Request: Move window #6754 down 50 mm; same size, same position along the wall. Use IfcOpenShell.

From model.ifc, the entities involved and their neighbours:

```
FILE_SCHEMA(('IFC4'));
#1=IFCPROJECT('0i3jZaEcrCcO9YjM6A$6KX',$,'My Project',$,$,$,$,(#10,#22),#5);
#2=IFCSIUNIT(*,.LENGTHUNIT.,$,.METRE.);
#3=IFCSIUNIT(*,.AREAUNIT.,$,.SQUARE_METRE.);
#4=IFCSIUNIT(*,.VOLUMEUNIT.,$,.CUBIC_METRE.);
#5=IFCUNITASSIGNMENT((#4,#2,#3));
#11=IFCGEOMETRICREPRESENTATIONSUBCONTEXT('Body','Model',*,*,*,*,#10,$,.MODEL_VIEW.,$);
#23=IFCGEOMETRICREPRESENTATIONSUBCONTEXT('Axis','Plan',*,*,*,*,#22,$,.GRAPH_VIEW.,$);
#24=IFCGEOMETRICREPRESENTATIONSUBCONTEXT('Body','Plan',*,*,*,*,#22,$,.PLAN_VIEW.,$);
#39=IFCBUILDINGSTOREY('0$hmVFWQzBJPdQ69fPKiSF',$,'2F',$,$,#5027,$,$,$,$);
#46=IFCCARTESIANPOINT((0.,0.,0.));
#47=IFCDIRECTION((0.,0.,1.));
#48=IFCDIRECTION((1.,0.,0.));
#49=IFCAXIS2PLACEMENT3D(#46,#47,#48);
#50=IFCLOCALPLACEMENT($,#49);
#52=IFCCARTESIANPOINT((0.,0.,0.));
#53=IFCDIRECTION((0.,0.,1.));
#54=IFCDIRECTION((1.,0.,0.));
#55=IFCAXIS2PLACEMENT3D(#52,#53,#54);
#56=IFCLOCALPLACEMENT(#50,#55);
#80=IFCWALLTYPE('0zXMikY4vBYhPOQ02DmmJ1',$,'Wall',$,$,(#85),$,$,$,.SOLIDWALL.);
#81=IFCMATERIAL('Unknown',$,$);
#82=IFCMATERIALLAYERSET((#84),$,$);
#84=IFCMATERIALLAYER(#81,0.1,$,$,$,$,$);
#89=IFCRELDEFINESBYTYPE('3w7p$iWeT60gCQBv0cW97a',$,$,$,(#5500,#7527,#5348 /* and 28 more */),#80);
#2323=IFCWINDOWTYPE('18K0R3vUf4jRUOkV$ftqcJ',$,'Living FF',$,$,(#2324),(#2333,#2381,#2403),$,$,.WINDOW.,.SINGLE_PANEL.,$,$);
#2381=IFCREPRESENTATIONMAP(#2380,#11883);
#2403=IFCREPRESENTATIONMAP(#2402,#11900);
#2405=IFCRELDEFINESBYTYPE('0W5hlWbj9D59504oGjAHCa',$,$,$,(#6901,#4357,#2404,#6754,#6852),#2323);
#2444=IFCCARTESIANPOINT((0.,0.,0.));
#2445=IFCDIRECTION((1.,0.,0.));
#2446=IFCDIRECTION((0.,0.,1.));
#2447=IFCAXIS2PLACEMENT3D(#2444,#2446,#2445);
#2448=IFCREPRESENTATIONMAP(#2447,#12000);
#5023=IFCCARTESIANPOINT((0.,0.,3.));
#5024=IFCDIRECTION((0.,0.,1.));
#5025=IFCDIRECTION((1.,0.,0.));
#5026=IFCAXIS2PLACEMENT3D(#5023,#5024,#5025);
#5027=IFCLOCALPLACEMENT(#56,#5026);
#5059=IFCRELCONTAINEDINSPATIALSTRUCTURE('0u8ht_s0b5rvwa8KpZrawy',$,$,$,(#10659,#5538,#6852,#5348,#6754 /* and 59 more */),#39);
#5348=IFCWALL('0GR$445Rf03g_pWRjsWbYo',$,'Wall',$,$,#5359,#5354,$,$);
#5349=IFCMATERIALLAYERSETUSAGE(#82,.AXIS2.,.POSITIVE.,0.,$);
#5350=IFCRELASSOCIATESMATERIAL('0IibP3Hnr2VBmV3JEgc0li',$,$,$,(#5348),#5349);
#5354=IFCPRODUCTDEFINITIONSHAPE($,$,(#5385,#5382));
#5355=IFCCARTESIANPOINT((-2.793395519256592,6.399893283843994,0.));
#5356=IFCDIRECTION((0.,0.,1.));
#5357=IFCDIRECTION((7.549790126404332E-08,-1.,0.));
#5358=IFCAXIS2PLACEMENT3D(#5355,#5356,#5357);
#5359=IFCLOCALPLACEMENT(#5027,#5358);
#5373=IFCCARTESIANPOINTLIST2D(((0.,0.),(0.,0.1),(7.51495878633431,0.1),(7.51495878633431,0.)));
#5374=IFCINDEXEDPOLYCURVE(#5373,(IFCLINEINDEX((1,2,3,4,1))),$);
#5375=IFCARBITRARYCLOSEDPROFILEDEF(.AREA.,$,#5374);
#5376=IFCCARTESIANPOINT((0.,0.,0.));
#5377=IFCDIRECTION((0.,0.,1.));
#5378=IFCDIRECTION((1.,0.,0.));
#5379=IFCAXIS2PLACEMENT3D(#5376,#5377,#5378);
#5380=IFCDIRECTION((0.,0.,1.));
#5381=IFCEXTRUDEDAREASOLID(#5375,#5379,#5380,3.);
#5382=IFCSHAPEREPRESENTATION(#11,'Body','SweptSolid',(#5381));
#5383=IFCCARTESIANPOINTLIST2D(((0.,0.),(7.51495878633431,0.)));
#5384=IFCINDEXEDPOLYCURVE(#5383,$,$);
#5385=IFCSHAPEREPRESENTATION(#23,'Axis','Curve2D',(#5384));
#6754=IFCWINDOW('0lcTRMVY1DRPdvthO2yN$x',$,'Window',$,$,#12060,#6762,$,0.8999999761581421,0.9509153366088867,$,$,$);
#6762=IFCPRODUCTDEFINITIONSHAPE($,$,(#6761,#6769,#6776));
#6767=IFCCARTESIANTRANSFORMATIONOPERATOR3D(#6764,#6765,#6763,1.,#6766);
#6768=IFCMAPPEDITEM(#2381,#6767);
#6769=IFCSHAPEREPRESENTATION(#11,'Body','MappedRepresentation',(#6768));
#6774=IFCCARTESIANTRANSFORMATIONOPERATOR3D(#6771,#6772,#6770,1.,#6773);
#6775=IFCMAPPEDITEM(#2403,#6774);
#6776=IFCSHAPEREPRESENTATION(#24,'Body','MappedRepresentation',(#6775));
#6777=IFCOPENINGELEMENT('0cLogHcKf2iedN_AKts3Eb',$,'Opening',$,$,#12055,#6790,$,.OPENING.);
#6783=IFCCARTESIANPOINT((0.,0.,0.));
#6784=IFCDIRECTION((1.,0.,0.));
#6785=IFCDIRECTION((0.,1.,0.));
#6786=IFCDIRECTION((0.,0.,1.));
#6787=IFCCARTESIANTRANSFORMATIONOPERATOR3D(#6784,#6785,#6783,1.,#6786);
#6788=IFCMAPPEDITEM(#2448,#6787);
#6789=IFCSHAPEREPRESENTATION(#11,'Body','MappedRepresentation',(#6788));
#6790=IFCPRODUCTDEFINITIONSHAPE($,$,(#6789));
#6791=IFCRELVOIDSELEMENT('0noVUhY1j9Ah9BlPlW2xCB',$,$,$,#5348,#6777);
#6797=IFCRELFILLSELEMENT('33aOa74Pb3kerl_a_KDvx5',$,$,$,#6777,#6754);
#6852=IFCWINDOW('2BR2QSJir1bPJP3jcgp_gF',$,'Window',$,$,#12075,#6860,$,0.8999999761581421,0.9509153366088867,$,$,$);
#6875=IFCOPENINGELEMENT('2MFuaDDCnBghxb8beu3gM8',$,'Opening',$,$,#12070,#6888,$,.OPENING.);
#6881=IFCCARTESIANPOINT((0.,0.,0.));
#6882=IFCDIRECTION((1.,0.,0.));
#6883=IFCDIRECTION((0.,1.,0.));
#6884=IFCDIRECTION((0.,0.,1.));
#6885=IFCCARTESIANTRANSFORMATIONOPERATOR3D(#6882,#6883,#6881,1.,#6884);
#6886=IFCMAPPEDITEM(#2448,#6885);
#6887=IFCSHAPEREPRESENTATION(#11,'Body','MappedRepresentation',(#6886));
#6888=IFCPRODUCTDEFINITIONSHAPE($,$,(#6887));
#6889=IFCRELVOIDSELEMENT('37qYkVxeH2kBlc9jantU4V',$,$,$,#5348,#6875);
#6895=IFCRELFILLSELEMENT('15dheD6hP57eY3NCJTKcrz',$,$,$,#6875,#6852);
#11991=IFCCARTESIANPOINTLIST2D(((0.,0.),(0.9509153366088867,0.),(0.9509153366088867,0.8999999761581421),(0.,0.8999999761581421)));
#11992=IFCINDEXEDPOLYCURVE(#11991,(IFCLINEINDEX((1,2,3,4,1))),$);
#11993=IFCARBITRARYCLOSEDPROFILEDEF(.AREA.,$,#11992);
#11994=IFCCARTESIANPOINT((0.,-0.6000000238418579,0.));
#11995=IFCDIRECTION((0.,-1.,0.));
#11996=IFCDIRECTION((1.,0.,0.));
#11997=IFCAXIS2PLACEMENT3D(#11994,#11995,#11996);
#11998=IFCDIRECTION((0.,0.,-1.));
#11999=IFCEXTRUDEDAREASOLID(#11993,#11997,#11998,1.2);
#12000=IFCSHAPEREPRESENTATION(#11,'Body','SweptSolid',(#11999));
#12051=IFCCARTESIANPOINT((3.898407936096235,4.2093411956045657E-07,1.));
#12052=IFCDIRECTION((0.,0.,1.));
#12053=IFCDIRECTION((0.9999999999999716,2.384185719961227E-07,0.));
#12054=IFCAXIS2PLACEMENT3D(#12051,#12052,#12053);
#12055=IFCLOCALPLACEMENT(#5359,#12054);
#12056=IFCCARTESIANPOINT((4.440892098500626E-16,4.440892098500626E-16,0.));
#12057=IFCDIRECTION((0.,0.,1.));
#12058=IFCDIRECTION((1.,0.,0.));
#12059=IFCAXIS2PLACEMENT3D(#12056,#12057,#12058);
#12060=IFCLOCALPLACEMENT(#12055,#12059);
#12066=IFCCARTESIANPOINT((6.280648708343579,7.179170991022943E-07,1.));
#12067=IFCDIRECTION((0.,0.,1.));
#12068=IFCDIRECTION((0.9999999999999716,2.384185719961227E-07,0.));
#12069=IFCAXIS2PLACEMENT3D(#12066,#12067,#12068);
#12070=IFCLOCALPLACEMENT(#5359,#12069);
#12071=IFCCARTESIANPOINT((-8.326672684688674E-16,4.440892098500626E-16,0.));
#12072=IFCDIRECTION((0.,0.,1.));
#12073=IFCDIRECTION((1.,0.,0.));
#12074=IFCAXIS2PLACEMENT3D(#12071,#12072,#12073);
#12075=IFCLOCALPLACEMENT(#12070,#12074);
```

```python
import numpy as np
import ifcopenshell
import ifcopenshell.api.geometry
import ifcopenshell.util.placement
import ifcopenshell.util.unit

model = ifcopenshell.open("model.ifc")
unit_scale = ifcopenshell.util.unit.calculate_unit_scale(model)

window = model.by_guid("0lcTRMVY1DRPdvthO2yN$x")
opening = window.FillsVoids[0].RelatingOpeningElement
dz = -0.05

shift = np.array([0.0, 0.0, dz])
# The window is placed relative to its opening, so it follows when the opening moves.
matrix = ifcopenshell.util.placement.get_local_placement(opening.ObjectPlacement)
matrix[:3, 3] += shift
ifcopenshell.api.geometry.edit_object_placement(
    model, product=opening, matrix=matrix, is_si=False, should_transform_children=True
)

print(f"moved by {dz * unit_scale:+.3f} m")

model.write("model_updated.ifc")
```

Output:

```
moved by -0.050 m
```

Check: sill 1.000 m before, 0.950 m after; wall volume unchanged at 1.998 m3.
